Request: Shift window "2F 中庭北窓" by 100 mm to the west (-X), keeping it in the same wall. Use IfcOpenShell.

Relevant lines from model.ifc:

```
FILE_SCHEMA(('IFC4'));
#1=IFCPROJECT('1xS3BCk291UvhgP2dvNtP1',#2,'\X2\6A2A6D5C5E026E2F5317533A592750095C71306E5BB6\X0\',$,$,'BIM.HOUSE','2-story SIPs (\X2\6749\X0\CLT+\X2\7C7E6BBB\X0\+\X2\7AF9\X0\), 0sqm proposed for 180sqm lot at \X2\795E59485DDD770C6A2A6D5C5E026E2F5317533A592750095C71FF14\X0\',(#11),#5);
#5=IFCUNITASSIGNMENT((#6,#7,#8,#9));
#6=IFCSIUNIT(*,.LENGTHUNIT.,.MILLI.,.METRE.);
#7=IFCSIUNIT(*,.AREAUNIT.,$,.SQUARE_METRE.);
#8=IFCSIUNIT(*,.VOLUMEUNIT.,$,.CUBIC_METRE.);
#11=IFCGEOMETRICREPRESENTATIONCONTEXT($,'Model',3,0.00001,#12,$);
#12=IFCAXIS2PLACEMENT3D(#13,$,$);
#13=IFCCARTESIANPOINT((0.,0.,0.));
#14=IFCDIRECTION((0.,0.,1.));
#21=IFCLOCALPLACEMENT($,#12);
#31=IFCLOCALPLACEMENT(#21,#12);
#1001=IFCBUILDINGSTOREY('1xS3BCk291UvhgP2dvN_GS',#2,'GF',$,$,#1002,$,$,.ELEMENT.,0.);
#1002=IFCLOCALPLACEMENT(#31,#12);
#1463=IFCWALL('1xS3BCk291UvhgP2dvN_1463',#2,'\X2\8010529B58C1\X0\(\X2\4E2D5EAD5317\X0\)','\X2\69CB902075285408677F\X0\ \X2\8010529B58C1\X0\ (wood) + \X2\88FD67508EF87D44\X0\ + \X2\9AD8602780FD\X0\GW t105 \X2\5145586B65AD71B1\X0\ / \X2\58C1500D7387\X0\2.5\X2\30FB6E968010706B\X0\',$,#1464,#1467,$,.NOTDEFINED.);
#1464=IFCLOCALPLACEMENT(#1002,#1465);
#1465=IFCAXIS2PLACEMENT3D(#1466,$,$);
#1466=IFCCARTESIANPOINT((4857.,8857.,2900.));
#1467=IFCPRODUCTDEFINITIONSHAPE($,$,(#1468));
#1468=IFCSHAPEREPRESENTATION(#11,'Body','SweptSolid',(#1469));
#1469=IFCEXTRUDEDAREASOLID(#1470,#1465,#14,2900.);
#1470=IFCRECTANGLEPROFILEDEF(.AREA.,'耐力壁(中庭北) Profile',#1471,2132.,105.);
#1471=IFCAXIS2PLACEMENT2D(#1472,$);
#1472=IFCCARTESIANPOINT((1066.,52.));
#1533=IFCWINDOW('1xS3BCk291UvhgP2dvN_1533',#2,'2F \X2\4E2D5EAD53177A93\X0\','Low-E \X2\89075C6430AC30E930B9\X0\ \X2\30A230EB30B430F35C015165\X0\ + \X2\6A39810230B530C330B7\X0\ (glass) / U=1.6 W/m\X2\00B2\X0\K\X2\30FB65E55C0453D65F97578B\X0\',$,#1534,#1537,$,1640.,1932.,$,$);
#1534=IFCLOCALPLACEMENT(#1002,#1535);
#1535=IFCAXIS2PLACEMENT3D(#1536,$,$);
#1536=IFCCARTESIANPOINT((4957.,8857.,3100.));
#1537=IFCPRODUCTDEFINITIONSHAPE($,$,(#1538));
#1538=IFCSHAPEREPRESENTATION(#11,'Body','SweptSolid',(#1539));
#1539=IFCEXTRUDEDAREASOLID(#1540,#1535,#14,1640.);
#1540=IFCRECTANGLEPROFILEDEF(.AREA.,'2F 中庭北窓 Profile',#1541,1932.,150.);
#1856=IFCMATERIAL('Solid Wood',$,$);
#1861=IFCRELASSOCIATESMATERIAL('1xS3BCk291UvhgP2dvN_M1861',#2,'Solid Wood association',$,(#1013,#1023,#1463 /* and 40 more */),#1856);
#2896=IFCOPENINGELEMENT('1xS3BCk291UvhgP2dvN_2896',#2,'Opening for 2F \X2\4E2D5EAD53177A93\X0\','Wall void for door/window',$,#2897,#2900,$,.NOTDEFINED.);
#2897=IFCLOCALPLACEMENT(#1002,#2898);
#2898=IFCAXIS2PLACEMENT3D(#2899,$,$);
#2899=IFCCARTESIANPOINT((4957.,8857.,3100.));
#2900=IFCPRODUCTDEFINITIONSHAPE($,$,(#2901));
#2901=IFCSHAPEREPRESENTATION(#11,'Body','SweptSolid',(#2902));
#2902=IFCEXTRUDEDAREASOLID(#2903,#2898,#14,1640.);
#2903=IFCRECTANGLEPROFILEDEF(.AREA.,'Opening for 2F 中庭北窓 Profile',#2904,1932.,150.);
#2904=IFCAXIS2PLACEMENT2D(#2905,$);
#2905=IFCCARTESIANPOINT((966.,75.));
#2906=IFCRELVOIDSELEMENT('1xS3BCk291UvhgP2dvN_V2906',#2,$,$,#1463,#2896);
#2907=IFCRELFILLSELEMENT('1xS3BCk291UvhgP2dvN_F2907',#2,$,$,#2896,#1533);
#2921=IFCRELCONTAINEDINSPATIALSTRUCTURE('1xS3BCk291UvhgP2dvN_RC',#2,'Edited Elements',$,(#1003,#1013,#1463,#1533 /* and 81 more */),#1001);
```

```python
import ifcopenshell
import ifcopenshell.api.geometry
import ifcopenshell.util.placement

model = ifcopenshell.open("model.ifc")

window = model.by_guid("1xS3BCk291UvhgP2dvN_1533")
opening = window.FillsVoids[0].RelatingOpeningElement
wall = opening.VoidsElements[0].RelatingBuildingElement

wall_matrix = ifcopenshell.util.placement.get_local_placement(wall.ObjectPlacement)
shift = wall_matrix[:3, 0] * -100.0
before = ifcopenshell.util.placement.get_local_placement(window.ObjectPlacement)[:3, 3].copy()

# The window is not placed relative to its opening, so move both.
for product in (opening, window):
    matrix = ifcopenshell.util.placement.get_local_placement(product.ObjectPlacement)
    matrix[:3, 3] += shift
    ifcopenshell.api.geometry.edit_object_placement(model, product=product, matrix=matrix, is_si=False)

after = ifcopenshell.util.placement.get_local_placement(window.ObjectPlacement)[:3, 3]
print("window moved by", (after - before).round(3) + 0.0)

model.write("model_updated.ifc")
```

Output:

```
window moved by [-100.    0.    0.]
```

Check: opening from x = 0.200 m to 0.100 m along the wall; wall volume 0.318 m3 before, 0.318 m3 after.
